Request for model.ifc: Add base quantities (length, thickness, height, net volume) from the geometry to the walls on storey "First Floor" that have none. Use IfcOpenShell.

First a look at what the model holds.

```python
import ifcopenshell
import ifcopenshell.util.element
import ifcopenshell.util.unit

model = ifcopenshell.open("model.ifc")
print(model.schema)
for unit_type in ("LENGTHUNIT", "AREAUNIT", "VOLUMEUNIT"):
    print(unit_type, ifcopenshell.util.unit.calculate_unit_scale(model, unit_type))
storey = next(s for s in model.by_type("IfcBuildingStorey") if s.Name == "First Floor")
walls = [e for e in ifcopenshell.util.element.get_decomposition(storey) if e.is_a("IfcWall")]
for e in sorted(walls, key=lambda e: e.id()):
    print(e.id(), e.is_a(), e.Name, list(ifcopenshell.util.element.get_psets(e, qtos_only=True)), sep=" | ")
```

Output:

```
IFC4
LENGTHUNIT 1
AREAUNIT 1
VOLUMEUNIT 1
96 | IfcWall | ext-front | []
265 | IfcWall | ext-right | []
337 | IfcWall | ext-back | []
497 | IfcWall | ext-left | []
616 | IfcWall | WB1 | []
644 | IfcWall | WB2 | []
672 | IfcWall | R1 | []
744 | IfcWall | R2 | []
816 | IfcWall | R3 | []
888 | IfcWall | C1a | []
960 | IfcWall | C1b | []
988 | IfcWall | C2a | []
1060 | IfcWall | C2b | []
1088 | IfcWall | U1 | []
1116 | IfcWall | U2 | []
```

```python
import ifcopenshell
import ifcopenshell.api.pset
import ifcopenshell.geom
import ifcopenshell.util.element
import ifcopenshell.util.shape
import ifcopenshell.util.unit

model = ifcopenshell.open("model.ifc")
unit_scale = ifcopenshell.util.unit.calculate_unit_scale(model)
volume_scale = ifcopenshell.util.unit.calculate_unit_scale(model, "VOLUMEUNIT")
settings = ifcopenshell.geom.settings()

storey = next(s for s in model.by_type("IfcBuildingStorey") if s.Name == "First Floor")
walls = [e for e in ifcopenshell.util.element.get_decomposition(storey) if e.is_a("IfcWall")]

for e in sorted(walls, key=lambda e: e.id()):
    if ifcopenshell.util.element.get_psets(e, qtos_only=True, should_inherit=False):
        continue
    # Geometry comes back in metres, in the element's own axes.
    shape = ifcopenshell.geom.create_shape(settings, e)
    values = {
        "Length": ifcopenshell.util.shape.get_x(shape.geometry) / unit_scale,
        "Width": ifcopenshell.util.shape.get_y(shape.geometry) / unit_scale,
        "Height": ifcopenshell.util.shape.get_z(shape.geometry) / unit_scale,
        "NetVolume": ifcopenshell.util.shape.get_volume(shape.geometry) / volume_scale,
    }
    qto = ifcopenshell.api.pset.add_qto(model, product=e, name="Qto_WallBaseQuantities")
    ifcopenshell.api.pset.edit_qto(model, qto=qto, properties=values)
    print(e.id(), {k: round(v, 3) for k, v in values.items()})

model.write("model_updated.ifc")
```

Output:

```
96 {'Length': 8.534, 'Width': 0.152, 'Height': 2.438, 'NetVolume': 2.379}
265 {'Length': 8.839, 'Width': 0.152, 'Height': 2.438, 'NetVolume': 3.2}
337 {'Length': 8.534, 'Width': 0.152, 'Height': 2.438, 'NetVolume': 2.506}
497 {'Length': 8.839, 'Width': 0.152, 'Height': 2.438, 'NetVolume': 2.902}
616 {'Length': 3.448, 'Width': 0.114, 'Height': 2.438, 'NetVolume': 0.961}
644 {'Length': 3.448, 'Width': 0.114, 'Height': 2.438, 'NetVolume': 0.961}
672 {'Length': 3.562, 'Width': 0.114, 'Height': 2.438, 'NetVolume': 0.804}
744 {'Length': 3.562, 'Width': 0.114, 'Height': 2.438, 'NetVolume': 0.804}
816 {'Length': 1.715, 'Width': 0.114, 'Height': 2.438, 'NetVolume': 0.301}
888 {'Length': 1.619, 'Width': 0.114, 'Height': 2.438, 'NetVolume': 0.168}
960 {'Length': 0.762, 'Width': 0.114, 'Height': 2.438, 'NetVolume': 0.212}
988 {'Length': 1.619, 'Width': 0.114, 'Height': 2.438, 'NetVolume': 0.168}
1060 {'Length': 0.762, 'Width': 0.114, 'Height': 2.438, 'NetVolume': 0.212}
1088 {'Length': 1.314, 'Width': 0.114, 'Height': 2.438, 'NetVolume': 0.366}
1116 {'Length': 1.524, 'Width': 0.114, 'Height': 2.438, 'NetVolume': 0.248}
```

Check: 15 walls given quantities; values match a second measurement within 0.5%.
